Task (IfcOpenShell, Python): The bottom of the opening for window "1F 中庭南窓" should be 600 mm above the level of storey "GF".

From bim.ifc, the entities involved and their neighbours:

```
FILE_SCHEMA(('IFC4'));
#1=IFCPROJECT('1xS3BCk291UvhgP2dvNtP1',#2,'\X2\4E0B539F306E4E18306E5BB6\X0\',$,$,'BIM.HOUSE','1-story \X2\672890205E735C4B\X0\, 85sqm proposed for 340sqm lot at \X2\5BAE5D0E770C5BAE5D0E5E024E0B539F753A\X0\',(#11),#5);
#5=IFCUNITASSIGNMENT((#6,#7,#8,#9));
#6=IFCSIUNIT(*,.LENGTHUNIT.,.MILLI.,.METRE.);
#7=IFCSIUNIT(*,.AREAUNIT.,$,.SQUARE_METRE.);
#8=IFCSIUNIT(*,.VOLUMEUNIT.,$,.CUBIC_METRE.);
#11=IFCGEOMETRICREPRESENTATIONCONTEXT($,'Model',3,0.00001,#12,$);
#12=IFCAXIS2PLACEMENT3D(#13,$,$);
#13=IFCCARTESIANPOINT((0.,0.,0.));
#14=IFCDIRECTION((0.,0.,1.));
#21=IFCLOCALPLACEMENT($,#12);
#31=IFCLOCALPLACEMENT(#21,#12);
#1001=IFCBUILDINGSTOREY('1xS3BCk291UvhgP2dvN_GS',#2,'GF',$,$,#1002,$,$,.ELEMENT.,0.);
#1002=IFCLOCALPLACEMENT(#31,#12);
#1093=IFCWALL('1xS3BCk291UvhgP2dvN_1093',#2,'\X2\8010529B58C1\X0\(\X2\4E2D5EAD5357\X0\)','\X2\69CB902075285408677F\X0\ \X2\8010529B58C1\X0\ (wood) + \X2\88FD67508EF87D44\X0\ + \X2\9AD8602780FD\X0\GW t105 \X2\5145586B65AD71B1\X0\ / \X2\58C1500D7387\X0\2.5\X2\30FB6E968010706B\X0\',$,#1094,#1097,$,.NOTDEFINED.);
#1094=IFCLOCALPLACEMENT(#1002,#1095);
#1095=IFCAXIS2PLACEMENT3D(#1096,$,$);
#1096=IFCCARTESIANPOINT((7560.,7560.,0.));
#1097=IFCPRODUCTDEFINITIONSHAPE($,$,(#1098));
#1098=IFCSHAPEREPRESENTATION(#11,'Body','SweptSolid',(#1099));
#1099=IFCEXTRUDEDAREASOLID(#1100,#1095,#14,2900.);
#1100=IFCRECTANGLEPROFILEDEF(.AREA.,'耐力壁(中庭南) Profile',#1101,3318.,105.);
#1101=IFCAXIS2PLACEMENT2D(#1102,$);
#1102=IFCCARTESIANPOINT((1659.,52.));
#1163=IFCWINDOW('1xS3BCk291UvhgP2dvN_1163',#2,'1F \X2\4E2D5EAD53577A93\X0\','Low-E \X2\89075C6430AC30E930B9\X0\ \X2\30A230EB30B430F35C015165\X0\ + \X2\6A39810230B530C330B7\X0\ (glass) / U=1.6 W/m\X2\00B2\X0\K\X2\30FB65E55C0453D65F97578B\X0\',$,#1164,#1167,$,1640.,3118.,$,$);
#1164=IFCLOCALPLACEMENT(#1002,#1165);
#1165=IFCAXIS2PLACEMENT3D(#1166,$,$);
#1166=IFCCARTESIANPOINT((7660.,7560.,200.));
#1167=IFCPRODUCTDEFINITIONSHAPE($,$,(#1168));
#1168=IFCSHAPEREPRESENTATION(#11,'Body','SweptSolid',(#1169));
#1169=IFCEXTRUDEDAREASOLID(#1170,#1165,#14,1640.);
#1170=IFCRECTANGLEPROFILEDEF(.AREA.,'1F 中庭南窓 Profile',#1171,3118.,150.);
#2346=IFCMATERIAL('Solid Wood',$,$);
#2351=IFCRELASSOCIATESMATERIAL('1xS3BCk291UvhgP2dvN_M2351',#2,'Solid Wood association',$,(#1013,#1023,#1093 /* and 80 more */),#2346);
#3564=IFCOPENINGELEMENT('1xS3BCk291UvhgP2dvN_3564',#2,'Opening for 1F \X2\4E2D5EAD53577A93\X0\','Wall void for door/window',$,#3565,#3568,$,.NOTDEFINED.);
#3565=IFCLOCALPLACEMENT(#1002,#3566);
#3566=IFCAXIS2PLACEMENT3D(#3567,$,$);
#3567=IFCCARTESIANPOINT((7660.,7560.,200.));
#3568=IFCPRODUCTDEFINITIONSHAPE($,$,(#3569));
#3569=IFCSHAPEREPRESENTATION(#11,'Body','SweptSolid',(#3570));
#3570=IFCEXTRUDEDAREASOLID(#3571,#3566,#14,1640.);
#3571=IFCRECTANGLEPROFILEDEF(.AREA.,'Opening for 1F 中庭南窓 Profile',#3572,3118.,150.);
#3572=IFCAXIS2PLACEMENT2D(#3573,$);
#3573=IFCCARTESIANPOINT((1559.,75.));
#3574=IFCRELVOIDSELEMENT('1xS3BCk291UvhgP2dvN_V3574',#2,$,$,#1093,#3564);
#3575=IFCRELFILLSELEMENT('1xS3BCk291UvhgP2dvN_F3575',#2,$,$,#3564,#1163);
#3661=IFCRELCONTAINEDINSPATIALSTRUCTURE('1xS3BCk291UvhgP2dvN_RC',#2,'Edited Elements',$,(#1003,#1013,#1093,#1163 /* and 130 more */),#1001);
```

```python
import numpy as np
import ifcopenshell
import ifcopenshell.api.geometry
import ifcopenshell.geom
import ifcopenshell.util.element
import ifcopenshell.util.placement
import ifcopenshell.util.shape
import ifcopenshell.util.unit

model = ifcopenshell.open("bim.ifc")
unit_scale = ifcopenshell.util.unit.calculate_unit_scale(model)

window = model.by_guid("1xS3BCk291UvhgP2dvN_1163")
opening = window.FillsVoids[0].RelatingOpeningElement
storey = ifcopenshell.util.element.get_container(window, ifc_class="IfcBuildingStorey")
level = ifcopenshell.util.placement.get_local_placement(storey.ObjectPlacement)[2, 3]

# The opening's origin need not be at the sill, so measure its lowest point.
shape = ifcopenshell.geom.create_shape(ifcopenshell.geom.settings(), opening)
bottom = ifcopenshell.util.shape.get_shape_bottom_elevation(shape, shape.geometry) / unit_scale
dz = level + 0.6 / unit_scale - bottom

shift = np.array([0.0, 0.0, dz])
# The window is not placed relative to its opening, so move both.
for product in (opening, window):
    matrix = ifcopenshell.util.placement.get_local_placement(product.ObjectPlacement)
    matrix[:3, 3] += shift
    ifcopenshell.api.geometry.edit_object_placement(model, product=product, matrix=matrix, is_si=False)

print(f"moved by {dz * unit_scale:+.3f} m")

model.write("bim_edited.ifc")
```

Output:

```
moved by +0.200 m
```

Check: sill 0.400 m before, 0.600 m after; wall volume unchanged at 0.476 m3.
